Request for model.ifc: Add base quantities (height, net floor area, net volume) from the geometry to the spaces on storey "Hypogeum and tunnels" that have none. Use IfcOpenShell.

First a look at what the model holds.

```python
import ifcopenshell
import ifcopenshell.util.element
import ifcopenshell.util.unit

model = ifcopenshell.open("model.ifc")
print(model.schema)
for unit_type in ("LENGTHUNIT", "AREAUNIT", "VOLUMEUNIT"):
    print(unit_type, ifcopenshell.util.unit.calculate_unit_scale(model, unit_type))
storey = next(s for s in model.by_type("IfcBuildingStorey") if s.Name == "Hypogeum and tunnels")
spaces = [e for e in ifcopenshell.util.element.get_decomposition(storey) if e.is_a("IfcSpace")]
for e in sorted(spaces, key=lambda e: e.id()):
    print(e.id(), e.is_a(), e.Name, list(ifcopenshell.util.element.get_psets(e, qtos_only=True)), sep=" | ")
```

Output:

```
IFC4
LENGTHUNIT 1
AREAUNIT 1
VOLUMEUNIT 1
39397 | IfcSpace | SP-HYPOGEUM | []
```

```python
import ifcopenshell
import ifcopenshell.api.pset
import ifcopenshell.geom
import ifcopenshell.util.element
import ifcopenshell.util.shape
import ifcopenshell.util.unit

model = ifcopenshell.open("model.ifc")
unit_scale = ifcopenshell.util.unit.calculate_unit_scale(model)
area_scale = ifcopenshell.util.unit.calculate_unit_scale(model, "AREAUNIT")
volume_scale = ifcopenshell.util.unit.calculate_unit_scale(model, "VOLUMEUNIT")
settings = ifcopenshell.geom.settings()

storey = next(s for s in model.by_type("IfcBuildingStorey") if s.Name == "Hypogeum and tunnels")
spaces = [e for e in ifcopenshell.util.element.get_decomposition(storey) if e.is_a("IfcSpace")]

for e in sorted(spaces, key=lambda e: e.id()):
    if ifcopenshell.util.element.get_psets(e, qtos_only=True, should_inherit=False):
        continue
    # Geometry comes back in metres, in the element's own axes.
    shape = ifcopenshell.geom.create_shape(settings, e)
    values = {
        "Height": ifcopenshell.util.shape.get_z(shape.geometry) / unit_scale,
        "NetFloorArea": ifcopenshell.util.shape.get_footprint_area(shape.geometry) / area_scale,
        "NetVolume": ifcopenshell.util.shape.get_volume(shape.geometry) / volume_scale,
    }
    qto = ifcopenshell.api.pset.add_qto(model, product=e, name="Qto_SpaceBaseQuantities")
    ifcopenshell.api.pset.edit_qto(model, qto=qto, properties=values)
    print(e.id(), {k: round(v, 3) for k, v in values.items()})

model.write("model_edited.ifc")
```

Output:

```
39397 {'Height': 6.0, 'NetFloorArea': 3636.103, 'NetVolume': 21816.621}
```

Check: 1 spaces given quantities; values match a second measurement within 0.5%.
